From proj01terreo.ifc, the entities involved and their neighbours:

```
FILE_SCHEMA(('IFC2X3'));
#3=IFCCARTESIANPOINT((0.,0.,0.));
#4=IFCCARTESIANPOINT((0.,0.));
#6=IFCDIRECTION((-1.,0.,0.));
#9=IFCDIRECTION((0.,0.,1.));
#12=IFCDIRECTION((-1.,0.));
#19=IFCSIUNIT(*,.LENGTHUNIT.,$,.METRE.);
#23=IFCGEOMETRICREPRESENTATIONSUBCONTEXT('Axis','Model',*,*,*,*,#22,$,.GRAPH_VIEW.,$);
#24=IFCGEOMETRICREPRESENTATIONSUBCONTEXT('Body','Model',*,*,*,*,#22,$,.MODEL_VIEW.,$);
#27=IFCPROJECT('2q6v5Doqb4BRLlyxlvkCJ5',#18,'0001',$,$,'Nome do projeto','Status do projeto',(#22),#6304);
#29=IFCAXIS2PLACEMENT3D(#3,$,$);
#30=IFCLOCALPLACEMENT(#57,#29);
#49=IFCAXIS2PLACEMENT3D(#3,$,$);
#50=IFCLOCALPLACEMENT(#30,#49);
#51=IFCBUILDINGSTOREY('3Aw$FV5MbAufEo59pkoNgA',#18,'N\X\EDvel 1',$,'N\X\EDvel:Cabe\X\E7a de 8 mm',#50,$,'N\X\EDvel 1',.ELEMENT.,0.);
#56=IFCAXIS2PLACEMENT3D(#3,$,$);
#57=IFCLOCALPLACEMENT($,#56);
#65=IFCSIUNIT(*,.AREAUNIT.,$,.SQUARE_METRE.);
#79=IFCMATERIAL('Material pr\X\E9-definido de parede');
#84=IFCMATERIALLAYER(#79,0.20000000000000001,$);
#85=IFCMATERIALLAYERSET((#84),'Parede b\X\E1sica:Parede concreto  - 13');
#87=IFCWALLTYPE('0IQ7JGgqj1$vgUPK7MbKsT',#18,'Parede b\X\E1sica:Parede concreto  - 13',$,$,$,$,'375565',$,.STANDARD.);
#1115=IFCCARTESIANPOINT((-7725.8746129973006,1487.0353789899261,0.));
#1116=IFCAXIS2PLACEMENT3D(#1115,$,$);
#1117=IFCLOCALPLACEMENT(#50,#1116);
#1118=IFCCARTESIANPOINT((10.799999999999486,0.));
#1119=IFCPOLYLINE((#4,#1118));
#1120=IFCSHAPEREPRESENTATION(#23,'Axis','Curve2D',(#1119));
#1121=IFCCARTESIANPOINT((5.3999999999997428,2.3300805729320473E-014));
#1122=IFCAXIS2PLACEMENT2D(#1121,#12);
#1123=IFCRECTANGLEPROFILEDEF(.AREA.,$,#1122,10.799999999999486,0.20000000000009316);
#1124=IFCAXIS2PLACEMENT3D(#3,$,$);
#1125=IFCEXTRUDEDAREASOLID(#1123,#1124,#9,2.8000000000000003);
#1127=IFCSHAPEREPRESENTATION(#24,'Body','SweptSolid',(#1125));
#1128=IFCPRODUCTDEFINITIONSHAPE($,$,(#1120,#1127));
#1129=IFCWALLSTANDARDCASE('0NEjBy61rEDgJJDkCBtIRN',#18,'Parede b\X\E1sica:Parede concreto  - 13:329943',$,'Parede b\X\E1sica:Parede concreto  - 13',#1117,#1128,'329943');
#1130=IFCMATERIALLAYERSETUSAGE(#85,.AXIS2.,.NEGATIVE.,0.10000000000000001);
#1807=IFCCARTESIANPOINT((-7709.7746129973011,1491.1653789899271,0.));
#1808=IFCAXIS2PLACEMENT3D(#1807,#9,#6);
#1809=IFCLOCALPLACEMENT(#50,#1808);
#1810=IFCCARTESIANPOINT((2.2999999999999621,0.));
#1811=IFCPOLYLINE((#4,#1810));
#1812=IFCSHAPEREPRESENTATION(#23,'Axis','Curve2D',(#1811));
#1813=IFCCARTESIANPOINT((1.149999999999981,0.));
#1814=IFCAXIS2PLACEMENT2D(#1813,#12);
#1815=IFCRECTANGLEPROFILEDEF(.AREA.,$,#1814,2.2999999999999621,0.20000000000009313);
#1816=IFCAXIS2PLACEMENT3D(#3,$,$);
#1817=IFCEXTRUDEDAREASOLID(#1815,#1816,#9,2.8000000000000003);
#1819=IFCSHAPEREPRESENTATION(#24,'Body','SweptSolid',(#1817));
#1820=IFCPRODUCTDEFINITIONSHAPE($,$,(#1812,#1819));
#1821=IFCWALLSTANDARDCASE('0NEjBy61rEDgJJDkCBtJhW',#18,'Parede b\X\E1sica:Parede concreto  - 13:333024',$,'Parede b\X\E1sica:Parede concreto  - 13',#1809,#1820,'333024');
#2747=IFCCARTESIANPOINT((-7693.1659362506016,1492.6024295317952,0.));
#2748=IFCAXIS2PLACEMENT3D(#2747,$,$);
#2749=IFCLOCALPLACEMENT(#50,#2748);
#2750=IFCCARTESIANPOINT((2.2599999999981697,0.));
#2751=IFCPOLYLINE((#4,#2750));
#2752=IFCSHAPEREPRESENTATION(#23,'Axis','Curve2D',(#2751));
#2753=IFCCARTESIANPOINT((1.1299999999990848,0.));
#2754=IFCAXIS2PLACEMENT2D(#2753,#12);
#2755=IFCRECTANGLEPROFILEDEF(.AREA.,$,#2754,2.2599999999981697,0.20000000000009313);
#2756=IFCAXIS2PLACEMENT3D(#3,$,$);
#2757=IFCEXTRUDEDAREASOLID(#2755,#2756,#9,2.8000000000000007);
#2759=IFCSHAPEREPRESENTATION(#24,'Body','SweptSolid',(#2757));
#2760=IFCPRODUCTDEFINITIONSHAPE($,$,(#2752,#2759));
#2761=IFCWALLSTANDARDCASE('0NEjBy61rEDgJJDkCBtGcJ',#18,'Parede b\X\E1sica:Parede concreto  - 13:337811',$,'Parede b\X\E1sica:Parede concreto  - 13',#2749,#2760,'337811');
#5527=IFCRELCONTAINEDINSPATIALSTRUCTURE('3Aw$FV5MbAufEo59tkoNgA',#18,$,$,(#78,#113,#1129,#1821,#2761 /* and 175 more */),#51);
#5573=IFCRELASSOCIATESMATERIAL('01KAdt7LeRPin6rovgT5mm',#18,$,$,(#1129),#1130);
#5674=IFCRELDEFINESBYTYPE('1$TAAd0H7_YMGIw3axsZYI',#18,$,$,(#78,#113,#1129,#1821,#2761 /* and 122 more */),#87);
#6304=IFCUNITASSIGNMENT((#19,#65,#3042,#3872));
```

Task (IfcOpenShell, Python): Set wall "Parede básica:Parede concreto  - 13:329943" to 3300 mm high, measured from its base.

```python
import ifcopenshell
import ifcopenshell.geom
import ifcopenshell.util.representation
import ifcopenshell.util.shape
import ifcopenshell.util.unit

model = ifcopenshell.open("proj01terreo.ifc")
unit_scale = ifcopenshell.util.unit.calculate_unit_scale(model)
settings = ifcopenshell.geom.settings()


def volume(element):
    """Net volume in cubic metres, openings subtracted."""
    shape = ifcopenshell.geom.create_shape(settings, element)
    return ifcopenshell.util.shape.get_volume(shape.geometry)


wall = model.by_id(1129)
before = volume(wall)

body = ifcopenshell.util.representation.get_representation(wall, "Model", "Body")
solid = body.Items[0]
old_height = solid.Depth
solid.Depth = 3.3 / unit_scale
after = volume(wall)

print(f"height {old_height:g} -> {solid.Depth:g}, volume {before:.3f} -> {after:.3f} m3")

model.write("proj01terreo-out.ifc")
```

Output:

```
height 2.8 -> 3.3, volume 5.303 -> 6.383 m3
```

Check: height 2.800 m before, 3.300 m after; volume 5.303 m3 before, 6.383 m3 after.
